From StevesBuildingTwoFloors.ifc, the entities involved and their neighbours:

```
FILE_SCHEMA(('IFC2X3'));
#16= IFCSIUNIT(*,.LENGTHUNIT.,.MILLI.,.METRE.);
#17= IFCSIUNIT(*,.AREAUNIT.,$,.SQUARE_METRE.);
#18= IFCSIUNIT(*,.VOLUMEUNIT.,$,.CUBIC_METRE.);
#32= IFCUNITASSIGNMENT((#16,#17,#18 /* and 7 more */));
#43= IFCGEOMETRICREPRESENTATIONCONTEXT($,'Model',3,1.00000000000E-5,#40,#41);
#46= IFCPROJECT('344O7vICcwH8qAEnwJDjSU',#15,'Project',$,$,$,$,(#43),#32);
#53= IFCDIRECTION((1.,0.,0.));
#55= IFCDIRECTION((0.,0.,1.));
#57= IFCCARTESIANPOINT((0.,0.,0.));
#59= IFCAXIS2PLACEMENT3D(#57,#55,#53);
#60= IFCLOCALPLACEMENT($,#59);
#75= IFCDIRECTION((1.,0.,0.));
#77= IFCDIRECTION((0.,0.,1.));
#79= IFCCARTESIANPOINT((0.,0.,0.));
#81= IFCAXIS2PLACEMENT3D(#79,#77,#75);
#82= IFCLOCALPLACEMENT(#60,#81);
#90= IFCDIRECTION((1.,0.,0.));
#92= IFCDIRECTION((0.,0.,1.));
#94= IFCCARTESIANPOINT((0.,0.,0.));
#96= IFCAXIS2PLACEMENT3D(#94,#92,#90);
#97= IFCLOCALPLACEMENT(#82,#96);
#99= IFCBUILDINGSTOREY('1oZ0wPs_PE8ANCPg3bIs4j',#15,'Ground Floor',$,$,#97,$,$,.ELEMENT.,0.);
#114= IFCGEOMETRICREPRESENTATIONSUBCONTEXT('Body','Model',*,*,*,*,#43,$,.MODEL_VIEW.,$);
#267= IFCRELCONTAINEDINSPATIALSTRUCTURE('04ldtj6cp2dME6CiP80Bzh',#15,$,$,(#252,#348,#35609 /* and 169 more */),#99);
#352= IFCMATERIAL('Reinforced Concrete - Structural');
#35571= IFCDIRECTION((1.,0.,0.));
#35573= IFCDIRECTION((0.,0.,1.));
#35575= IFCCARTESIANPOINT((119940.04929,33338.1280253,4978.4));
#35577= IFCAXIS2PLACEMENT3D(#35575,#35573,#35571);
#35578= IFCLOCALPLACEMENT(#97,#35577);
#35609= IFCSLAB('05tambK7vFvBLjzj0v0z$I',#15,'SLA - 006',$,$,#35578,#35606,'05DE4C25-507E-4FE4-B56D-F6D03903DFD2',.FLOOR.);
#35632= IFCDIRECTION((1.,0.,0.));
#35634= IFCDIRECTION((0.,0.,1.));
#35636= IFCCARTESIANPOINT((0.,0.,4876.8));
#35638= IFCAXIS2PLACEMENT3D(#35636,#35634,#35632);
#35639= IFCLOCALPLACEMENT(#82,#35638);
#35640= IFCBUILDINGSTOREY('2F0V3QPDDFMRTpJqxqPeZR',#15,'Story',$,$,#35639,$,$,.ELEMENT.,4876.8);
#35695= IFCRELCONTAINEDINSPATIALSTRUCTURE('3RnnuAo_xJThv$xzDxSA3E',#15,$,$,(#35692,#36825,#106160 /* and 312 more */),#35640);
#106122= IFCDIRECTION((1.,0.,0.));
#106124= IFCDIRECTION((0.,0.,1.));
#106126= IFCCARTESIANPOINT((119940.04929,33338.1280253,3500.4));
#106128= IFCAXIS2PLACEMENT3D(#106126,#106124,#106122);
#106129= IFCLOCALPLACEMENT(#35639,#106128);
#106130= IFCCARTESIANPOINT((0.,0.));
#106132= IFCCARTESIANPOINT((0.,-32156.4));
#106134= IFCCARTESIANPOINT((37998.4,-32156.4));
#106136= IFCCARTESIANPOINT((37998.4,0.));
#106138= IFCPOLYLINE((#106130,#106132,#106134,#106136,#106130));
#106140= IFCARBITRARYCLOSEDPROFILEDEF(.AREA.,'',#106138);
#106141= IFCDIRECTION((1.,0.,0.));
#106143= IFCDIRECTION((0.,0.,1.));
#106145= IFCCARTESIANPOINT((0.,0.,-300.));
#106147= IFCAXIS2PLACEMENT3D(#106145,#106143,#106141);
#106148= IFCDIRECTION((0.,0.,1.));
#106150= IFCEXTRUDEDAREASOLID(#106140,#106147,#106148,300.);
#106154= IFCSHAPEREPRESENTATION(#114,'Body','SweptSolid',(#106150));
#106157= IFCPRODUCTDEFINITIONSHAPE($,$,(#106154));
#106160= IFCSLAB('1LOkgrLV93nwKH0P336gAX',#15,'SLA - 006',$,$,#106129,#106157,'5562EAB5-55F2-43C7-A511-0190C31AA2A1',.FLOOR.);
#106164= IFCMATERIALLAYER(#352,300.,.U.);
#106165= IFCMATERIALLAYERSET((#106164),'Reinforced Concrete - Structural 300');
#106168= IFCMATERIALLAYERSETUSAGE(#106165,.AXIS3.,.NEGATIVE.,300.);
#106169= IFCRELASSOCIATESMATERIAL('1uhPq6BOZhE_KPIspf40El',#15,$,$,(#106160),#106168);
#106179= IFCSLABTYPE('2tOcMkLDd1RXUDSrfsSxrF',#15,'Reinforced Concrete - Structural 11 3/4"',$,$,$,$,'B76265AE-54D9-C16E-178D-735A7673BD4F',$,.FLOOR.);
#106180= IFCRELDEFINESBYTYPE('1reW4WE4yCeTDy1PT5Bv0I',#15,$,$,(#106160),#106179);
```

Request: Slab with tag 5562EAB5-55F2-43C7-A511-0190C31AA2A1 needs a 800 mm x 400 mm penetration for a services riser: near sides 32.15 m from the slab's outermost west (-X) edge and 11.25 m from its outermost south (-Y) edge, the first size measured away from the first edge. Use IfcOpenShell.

```python
import numpy as np
import ifcopenshell
import ifcopenshell.api.feature
import ifcopenshell.api.geometry
import ifcopenshell.api.root
import ifcopenshell.geom
import ifcopenshell.util.placement
import ifcopenshell.util.representation
import ifcopenshell.util.shape
import ifcopenshell.util.unit

model = ifcopenshell.open("StevesBuildingTwoFloors.ifc")
unit_scale = ifcopenshell.util.unit.calculate_unit_scale(model)
settings = ifcopenshell.geom.settings()


def volume(element):
    """Net volume in cubic metres, openings subtracted."""
    shape = ifcopenshell.geom.create_shape(settings, element)
    return ifcopenshell.util.shape.get_volume(shape.geometry)


slab = model.by_guid("1LOkgrLV93nwKH0P336gAX")
before = volume(slab)

# Extent in the slab's own axes, in metres. The edges named are its -X and -Y sides.
slab_shape = ifcopenshell.geom.create_shape(settings, slab)
vertices = ifcopenshell.util.shape.get_vertices(slab_shape.geometry)
x_min, y_min, bottom = vertices.min(axis=0)
top = vertices[:, 2].max()

opening = ifcopenshell.api.root.create_entity(model, ifc_class="IfcOpeningElement", name="Services riser opening")
context = ifcopenshell.util.representation.get_context(model, "Model", "Body", "MODEL_VIEW")
width, depth = 0.8, 0.4
outline = [(0.0, 0.0), (width, 0.0), (width, depth), (0.0, depth), (0.0, 0.0)]
# Overshoot both faces by 50 mm so the cut is clean.
shape = ifcopenshell.api.geometry.add_slab_representation(
    model, context=context, depth=top - bottom + 0.1, polyline=outline
)
ifcopenshell.api.geometry.assign_representation(model, product=opening, representation=shape)

matrix = ifcopenshell.util.placement.get_local_placement(slab.ObjectPlacement)
matrix[:, 3] = matrix @ np.append(np.array([x_min + 32.15, y_min + 11.25, bottom - 0.05]) / unit_scale, 1.0)
ifcopenshell.api.geometry.edit_object_placement(model, product=opening, matrix=matrix, is_si=False)
ifcopenshell.api.feature.add_feature(model, feature=opening, element=slab)

after = volume(slab)

print(f"slab volume {before:.3f} -> {after:.3f} m3")

model.write("StevesBuildingTwoFloors_rev.ifc")
```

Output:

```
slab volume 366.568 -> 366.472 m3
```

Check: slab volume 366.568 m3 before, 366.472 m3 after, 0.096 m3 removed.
